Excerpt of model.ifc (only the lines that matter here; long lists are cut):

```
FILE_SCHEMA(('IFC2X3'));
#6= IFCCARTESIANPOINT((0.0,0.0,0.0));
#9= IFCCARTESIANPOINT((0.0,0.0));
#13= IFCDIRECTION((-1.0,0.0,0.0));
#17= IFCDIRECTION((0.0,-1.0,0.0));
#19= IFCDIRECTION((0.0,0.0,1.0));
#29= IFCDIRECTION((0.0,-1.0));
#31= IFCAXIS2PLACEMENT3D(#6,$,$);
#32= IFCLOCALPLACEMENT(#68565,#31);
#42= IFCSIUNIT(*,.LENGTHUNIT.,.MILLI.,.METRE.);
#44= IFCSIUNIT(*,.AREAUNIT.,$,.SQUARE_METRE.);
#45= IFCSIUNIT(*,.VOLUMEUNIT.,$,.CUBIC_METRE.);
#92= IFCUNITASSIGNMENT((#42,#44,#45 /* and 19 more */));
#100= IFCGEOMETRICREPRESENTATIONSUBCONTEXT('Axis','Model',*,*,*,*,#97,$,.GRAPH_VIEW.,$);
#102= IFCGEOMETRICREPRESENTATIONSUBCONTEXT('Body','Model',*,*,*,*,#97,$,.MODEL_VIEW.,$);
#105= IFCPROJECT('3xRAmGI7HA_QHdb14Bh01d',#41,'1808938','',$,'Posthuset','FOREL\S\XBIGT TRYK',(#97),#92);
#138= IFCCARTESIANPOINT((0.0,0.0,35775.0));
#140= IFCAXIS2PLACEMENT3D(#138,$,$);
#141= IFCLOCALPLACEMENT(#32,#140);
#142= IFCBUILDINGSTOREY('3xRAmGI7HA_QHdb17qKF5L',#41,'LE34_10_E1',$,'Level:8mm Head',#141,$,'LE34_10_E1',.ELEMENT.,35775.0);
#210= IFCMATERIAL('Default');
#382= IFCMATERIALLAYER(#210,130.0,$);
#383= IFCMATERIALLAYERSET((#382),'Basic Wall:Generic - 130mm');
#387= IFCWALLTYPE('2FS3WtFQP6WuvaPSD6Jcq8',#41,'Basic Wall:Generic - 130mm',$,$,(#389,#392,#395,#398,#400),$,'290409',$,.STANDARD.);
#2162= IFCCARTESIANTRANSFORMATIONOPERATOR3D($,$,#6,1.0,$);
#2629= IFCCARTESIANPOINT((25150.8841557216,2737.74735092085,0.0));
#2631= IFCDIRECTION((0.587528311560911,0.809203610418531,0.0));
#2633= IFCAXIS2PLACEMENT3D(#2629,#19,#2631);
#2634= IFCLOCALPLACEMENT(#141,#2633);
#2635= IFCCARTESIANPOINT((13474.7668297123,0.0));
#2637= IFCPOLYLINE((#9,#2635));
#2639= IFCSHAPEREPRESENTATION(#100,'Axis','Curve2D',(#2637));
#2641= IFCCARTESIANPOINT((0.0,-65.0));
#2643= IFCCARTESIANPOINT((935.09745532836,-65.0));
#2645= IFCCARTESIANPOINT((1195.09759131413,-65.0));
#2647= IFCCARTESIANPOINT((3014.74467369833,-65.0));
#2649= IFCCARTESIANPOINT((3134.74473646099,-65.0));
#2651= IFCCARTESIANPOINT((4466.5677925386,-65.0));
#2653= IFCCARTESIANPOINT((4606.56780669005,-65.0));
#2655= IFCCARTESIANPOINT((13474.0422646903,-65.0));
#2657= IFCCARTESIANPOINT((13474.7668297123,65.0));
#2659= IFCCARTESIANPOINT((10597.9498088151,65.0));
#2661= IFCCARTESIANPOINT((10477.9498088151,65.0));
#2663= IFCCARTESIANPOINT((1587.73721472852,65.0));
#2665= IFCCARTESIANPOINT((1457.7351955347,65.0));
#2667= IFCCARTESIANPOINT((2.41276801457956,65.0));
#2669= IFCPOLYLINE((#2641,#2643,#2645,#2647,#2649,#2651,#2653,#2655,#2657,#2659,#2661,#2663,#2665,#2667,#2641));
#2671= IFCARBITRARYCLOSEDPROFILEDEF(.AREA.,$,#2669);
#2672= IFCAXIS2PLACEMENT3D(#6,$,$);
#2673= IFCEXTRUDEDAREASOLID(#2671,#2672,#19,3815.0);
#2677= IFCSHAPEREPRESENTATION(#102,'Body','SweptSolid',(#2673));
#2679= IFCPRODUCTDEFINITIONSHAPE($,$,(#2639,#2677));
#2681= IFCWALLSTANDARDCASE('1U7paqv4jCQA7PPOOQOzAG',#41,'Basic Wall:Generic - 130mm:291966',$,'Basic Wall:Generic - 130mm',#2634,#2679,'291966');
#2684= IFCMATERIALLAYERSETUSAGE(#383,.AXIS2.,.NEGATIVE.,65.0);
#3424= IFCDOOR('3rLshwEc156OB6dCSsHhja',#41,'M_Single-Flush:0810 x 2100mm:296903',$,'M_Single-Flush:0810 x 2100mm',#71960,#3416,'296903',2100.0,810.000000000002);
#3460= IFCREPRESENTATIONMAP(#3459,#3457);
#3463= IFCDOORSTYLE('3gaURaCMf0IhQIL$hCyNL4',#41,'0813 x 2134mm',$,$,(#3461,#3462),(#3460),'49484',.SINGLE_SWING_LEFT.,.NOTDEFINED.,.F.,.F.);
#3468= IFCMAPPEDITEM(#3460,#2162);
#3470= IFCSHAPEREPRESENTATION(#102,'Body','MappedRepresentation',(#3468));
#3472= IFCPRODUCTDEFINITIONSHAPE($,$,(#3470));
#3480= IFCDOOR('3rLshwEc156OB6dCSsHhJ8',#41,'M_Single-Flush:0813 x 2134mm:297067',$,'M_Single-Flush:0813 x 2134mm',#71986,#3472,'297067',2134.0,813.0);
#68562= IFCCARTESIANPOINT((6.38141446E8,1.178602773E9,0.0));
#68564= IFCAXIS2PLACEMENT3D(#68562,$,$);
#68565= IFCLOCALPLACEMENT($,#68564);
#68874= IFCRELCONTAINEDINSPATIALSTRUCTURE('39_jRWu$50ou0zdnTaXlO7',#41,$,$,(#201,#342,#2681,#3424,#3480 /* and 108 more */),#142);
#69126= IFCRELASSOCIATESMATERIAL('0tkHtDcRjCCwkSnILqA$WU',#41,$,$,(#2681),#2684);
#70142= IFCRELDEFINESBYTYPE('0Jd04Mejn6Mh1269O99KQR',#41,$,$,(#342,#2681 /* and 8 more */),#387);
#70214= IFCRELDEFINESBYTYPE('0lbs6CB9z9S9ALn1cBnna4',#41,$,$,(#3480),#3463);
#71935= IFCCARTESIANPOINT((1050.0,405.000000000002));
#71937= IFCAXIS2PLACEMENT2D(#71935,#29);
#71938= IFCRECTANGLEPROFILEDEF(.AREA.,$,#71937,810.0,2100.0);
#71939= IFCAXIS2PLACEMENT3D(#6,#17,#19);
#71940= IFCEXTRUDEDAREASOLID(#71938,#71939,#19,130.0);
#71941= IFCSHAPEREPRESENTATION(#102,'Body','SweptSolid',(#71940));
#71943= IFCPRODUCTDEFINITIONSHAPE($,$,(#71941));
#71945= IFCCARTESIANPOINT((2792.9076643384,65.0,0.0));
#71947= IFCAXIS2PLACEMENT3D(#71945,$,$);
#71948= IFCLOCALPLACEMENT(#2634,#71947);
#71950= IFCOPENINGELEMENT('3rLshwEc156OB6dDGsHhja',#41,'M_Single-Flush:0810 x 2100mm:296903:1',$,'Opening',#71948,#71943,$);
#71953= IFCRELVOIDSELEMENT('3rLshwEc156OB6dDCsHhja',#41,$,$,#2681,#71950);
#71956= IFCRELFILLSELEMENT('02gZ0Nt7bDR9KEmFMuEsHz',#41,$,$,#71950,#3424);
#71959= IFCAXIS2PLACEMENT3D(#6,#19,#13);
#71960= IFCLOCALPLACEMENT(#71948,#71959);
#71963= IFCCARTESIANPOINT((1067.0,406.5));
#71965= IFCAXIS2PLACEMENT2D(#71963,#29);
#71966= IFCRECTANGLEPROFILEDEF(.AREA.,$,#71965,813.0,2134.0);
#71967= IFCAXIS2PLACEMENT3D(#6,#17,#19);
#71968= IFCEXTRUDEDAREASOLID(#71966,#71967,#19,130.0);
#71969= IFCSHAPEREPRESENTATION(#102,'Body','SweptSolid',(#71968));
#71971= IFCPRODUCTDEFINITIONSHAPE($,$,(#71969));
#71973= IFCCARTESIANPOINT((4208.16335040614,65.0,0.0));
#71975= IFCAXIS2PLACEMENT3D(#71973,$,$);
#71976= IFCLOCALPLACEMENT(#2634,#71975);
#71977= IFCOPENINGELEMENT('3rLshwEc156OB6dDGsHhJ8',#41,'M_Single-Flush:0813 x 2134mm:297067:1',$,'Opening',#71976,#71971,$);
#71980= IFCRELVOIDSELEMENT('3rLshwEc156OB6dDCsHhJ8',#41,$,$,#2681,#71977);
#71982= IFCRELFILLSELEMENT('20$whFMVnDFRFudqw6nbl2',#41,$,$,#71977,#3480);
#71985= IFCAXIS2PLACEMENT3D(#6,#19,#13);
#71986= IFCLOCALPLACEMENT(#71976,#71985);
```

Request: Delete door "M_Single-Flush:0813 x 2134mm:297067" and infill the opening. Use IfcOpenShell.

```python
import ifcopenshell
import ifcopenshell.api.feature
import ifcopenshell.api.root
import ifcopenshell.geom
import ifcopenshell.util.shape

model = ifcopenshell.open("model.ifc")
settings = ifcopenshell.geom.settings()


def volume(element):
    """Net volume in cubic metres, openings subtracted."""
    shape = ifcopenshell.geom.create_shape(settings, element)
    return ifcopenshell.util.shape.get_volume(shape.geometry)


door = model.by_guid("3rLshwEc156OB6dCSsHhJ8")
opening = door.FillsVoids[0].RelatingOpeningElement
wall = opening.VoidsElements[0].RelatingBuildingElement
before = volume(wall)

ifcopenshell.api.root.remove_product(model, product=door)
ifcopenshell.api.feature.remove_feature(model, feature=opening)

after = volume(wall)

print(f"wall volume {before:.3f} -> {after:.3f} m3")

model.write("model_edited.ifc")
```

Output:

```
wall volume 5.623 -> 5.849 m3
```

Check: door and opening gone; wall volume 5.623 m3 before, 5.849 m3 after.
